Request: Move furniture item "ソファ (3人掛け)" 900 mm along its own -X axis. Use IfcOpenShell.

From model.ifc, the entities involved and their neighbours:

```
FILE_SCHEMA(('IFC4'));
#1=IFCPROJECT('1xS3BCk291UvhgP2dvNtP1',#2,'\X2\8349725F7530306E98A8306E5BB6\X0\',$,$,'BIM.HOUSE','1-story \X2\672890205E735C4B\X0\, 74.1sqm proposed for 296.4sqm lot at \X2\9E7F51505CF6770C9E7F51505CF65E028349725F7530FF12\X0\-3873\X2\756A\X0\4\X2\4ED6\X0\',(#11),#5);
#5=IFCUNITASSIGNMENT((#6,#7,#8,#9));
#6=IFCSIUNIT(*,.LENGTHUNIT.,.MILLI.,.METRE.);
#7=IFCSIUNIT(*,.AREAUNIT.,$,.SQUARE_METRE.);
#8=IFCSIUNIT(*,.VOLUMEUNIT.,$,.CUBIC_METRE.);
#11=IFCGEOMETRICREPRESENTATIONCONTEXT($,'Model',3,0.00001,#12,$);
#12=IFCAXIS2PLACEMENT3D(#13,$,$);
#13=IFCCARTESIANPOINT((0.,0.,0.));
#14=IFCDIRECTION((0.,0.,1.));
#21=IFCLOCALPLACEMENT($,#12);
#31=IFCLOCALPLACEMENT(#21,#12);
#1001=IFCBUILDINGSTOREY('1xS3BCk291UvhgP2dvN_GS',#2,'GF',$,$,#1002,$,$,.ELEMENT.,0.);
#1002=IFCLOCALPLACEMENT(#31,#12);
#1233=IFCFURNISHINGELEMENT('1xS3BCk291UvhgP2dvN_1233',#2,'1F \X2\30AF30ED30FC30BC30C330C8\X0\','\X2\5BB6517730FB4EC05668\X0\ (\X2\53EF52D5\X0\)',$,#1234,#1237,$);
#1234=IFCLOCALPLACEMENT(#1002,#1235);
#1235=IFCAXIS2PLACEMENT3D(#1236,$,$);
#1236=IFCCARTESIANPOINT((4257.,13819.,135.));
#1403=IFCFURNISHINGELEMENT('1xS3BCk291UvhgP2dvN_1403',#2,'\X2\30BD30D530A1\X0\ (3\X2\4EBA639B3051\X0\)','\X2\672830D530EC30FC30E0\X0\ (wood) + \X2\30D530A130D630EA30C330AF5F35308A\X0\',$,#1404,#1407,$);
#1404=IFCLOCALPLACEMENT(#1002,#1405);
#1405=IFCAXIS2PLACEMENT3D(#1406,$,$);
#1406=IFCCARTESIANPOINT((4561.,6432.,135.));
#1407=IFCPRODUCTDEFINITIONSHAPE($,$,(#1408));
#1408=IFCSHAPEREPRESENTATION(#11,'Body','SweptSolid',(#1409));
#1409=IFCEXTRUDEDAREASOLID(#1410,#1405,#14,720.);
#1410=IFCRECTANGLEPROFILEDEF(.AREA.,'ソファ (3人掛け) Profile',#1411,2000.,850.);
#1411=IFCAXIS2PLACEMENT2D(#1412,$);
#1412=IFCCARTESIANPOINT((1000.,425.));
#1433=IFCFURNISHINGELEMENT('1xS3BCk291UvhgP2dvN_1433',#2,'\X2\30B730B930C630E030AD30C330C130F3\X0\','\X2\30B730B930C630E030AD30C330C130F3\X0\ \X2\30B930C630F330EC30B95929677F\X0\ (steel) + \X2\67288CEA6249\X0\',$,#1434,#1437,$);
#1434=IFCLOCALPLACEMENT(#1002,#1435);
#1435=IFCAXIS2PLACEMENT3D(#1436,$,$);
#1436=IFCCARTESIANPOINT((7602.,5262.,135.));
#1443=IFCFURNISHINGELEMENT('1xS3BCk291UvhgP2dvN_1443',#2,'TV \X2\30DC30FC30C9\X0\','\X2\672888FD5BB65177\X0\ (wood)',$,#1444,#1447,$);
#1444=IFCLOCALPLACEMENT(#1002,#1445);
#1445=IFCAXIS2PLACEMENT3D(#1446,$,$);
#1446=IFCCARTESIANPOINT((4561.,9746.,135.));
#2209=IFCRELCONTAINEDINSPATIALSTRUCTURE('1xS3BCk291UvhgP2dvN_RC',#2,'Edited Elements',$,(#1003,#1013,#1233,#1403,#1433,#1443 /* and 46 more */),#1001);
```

```python
import ifcopenshell
import ifcopenshell.api.geometry
import ifcopenshell.util.placement

model = ifcopenshell.open("model.ifc")

item = model.by_guid("1xS3BCk291UvhgP2dvN_1403")
matrix = ifcopenshell.util.placement.get_local_placement(item.ObjectPlacement)
matrix[:3, 3] -= matrix[:3, 0] * 900.0
ifcopenshell.api.geometry.edit_object_placement(model, product=item, matrix=matrix, is_si=False)

print(ifcopenshell.util.placement.get_local_placement(item.ObjectPlacement).round(3) + 0.0)

model.write("model_updated.ifc")
```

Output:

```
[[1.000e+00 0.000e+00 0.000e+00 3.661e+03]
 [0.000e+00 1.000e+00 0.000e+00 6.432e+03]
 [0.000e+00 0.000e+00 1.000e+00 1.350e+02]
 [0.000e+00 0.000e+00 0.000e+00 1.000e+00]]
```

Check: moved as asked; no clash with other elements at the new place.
